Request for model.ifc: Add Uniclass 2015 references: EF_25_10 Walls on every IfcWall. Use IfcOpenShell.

First a look at what the model holds.

```python
import ifcopenshell

model = ifcopenshell.open("model.ifc")
print(model.schema)
print("classifications:", [c.Name for c in model.by_type("IfcClassification")])
for ifc_class in ("IfcDoor", "IfcRoof", "IfcStair", "IfcWall", "IfcWindow"):
    print(ifc_class, len(model.by_type(ifc_class)))
```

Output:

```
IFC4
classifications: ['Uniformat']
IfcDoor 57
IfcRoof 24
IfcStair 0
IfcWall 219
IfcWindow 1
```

```python
import ifcopenshell
import ifcopenshell.api.classification

model = ifcopenshell.open("model.ifc")

system = ifcopenshell.api.classification.add_classification(model, classification="Uniclass 2015")

codes = {
    "IfcWall": ("EF_25_10", "Walls"),
}
for ifc_class, (code, name) in codes.items():
    products = model.by_type(ifc_class)
    ifcopenshell.api.classification.add_reference(
        model, products=products, classification=system, identification=code, name=name
    )
    print(code, len(products))

model.write("model_edited.ifc")
```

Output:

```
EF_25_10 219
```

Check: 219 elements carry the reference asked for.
